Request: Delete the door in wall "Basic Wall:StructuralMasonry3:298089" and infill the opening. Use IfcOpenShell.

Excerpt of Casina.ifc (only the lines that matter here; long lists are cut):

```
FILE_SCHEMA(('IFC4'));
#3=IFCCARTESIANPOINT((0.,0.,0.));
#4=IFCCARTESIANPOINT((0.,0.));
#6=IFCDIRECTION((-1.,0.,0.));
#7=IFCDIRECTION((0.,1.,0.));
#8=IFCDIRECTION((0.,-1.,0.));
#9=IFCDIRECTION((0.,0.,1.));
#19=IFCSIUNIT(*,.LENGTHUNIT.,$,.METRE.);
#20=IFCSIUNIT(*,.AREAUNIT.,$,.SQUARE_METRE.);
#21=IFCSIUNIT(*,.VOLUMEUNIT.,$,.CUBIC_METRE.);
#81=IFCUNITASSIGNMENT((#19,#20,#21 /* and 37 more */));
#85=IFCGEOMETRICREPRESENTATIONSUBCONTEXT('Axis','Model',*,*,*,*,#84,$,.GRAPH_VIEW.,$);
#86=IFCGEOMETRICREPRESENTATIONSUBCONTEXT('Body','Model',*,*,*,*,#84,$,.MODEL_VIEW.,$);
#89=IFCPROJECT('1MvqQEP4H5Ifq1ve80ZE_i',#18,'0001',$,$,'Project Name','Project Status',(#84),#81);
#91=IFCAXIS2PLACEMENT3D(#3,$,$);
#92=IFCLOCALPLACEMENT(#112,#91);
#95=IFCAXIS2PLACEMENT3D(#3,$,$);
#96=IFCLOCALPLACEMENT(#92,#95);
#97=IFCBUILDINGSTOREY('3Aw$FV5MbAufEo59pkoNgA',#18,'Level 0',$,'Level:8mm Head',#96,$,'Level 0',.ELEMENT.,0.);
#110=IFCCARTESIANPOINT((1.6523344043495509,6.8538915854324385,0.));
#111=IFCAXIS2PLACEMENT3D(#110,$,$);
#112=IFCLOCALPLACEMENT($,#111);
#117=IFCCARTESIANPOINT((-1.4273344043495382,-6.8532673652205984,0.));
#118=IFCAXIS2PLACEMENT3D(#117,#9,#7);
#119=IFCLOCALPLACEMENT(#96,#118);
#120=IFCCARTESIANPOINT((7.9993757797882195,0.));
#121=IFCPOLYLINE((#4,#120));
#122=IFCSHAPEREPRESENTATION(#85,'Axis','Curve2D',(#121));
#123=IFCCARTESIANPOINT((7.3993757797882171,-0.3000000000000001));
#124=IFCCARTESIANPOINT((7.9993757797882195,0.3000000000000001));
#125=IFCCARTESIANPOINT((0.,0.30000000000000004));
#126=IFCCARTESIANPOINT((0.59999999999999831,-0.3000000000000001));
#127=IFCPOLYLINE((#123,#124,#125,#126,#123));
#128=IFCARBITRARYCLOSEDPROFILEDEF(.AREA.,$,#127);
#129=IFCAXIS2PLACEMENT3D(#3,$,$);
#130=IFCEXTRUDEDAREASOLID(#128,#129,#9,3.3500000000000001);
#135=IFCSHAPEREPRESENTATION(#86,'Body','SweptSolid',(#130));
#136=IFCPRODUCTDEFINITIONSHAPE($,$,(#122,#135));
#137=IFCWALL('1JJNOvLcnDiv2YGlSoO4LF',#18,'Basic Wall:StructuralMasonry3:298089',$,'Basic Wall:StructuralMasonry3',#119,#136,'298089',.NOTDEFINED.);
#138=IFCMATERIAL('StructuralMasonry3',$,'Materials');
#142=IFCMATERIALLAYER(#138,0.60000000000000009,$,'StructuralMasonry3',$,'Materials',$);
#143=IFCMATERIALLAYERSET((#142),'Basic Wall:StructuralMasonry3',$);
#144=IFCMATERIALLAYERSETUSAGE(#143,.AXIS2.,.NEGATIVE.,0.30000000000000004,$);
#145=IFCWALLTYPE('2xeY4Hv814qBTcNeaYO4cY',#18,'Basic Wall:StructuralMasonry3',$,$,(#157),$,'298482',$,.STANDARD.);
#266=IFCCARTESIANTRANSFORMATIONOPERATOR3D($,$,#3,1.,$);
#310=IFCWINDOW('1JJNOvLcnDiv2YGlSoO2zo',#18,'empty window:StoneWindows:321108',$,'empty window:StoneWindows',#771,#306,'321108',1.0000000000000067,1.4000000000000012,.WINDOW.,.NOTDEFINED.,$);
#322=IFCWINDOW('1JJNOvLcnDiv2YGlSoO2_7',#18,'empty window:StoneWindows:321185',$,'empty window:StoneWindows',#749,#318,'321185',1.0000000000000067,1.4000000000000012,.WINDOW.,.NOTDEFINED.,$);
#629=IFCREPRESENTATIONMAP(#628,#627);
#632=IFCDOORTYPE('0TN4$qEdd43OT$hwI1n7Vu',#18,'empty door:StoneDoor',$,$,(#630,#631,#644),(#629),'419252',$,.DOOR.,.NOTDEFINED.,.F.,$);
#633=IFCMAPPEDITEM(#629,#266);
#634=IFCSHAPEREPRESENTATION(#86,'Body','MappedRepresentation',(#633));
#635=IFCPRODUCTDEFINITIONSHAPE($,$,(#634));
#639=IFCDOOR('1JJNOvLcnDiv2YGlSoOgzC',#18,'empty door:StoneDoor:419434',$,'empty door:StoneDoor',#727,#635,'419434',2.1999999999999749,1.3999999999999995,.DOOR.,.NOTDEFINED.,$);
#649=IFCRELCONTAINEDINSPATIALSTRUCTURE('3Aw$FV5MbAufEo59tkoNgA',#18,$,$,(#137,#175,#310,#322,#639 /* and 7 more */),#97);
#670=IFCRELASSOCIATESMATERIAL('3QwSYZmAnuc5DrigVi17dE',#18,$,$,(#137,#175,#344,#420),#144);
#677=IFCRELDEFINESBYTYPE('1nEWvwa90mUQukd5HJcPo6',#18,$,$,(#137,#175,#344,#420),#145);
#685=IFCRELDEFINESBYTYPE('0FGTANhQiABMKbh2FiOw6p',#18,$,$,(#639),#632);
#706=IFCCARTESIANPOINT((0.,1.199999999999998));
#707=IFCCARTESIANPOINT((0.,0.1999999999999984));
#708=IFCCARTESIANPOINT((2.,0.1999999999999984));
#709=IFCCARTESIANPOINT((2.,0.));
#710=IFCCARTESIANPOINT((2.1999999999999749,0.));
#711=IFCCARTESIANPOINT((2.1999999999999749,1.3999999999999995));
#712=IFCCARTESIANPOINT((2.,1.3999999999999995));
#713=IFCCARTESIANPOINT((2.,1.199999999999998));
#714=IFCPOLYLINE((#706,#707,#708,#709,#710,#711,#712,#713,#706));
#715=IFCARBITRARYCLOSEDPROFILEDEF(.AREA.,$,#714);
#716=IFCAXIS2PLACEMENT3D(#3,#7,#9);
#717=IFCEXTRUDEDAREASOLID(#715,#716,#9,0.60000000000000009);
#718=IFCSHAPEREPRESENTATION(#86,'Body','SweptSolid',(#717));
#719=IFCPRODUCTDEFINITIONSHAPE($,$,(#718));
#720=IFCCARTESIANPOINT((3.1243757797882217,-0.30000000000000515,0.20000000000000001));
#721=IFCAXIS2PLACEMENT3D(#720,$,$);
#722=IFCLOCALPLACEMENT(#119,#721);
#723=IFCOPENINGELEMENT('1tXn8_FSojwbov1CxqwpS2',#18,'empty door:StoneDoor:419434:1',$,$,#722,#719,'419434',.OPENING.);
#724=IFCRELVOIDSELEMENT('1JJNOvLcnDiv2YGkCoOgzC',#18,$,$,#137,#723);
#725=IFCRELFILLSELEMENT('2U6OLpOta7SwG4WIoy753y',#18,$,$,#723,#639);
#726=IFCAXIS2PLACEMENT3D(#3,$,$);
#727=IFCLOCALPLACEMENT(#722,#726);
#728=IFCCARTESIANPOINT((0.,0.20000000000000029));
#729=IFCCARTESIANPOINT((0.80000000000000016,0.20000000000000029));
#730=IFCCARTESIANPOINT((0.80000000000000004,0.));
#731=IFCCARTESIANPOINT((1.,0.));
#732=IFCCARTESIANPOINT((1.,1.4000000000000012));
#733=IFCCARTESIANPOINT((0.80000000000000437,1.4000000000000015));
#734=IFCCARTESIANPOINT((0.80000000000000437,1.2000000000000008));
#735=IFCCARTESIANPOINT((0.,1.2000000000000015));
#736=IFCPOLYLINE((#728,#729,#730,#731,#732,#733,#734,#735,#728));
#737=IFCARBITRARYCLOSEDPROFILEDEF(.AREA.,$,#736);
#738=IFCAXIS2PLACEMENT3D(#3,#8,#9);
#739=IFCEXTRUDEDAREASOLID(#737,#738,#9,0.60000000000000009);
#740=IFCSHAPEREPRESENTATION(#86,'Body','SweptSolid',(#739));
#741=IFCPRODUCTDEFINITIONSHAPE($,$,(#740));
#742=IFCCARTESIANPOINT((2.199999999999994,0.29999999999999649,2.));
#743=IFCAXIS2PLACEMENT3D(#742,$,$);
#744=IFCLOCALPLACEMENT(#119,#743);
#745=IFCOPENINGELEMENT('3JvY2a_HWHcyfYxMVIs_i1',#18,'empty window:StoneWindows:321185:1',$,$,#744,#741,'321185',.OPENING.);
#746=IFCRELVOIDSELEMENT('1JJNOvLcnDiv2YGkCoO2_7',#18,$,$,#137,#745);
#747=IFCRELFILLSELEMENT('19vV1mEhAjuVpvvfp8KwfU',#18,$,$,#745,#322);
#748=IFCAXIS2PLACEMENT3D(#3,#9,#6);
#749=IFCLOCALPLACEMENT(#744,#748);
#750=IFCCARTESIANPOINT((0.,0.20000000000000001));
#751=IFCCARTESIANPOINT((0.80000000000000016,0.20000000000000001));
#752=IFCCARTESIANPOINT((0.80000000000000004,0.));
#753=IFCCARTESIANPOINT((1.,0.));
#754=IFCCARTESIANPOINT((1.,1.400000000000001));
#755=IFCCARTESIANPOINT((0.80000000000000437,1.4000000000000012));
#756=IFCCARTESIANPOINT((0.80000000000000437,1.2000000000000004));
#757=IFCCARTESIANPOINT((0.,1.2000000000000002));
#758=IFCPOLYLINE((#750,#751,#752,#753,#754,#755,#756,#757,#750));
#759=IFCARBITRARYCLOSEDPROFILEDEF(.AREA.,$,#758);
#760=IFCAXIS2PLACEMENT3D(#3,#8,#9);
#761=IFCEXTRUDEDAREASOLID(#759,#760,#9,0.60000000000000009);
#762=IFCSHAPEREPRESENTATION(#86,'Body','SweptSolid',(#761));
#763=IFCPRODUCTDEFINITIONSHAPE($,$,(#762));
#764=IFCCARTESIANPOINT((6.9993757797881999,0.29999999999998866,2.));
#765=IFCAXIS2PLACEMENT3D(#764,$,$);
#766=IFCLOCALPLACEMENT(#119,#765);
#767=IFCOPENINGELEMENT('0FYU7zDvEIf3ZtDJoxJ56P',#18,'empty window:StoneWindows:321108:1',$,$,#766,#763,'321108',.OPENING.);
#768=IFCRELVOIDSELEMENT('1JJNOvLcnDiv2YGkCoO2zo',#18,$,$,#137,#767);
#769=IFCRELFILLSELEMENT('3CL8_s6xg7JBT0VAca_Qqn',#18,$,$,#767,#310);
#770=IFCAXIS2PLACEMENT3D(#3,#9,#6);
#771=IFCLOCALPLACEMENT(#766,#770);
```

```python
import ifcopenshell
import ifcopenshell.api.feature
import ifcopenshell.api.root
import ifcopenshell.geom
import ifcopenshell.util.shape

model = ifcopenshell.open("Casina.ifc")
settings = ifcopenshell.geom.settings()


def volume(element):
    """Net volume in cubic metres, openings subtracted."""
    shape = ifcopenshell.geom.create_shape(settings, element)
    return ifcopenshell.util.shape.get_volume(shape.geometry)


door = model.by_guid("1JJNOvLcnDiv2YGlSoOgzC")
opening = door.FillsVoids[0].RelatingOpeningElement
wall = opening.VoidsElements[0].RelatingBuildingElement
before = volume(wall)

ifcopenshell.api.root.remove_product(model, product=door)
ifcopenshell.api.feature.remove_feature(model, feature=opening)

after = volume(wall)

print(f"wall volume {before:.3f} -> {after:.3f} m3")

model.write("Casina_updated.ifc")
```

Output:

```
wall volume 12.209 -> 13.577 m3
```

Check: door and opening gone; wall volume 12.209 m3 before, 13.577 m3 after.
